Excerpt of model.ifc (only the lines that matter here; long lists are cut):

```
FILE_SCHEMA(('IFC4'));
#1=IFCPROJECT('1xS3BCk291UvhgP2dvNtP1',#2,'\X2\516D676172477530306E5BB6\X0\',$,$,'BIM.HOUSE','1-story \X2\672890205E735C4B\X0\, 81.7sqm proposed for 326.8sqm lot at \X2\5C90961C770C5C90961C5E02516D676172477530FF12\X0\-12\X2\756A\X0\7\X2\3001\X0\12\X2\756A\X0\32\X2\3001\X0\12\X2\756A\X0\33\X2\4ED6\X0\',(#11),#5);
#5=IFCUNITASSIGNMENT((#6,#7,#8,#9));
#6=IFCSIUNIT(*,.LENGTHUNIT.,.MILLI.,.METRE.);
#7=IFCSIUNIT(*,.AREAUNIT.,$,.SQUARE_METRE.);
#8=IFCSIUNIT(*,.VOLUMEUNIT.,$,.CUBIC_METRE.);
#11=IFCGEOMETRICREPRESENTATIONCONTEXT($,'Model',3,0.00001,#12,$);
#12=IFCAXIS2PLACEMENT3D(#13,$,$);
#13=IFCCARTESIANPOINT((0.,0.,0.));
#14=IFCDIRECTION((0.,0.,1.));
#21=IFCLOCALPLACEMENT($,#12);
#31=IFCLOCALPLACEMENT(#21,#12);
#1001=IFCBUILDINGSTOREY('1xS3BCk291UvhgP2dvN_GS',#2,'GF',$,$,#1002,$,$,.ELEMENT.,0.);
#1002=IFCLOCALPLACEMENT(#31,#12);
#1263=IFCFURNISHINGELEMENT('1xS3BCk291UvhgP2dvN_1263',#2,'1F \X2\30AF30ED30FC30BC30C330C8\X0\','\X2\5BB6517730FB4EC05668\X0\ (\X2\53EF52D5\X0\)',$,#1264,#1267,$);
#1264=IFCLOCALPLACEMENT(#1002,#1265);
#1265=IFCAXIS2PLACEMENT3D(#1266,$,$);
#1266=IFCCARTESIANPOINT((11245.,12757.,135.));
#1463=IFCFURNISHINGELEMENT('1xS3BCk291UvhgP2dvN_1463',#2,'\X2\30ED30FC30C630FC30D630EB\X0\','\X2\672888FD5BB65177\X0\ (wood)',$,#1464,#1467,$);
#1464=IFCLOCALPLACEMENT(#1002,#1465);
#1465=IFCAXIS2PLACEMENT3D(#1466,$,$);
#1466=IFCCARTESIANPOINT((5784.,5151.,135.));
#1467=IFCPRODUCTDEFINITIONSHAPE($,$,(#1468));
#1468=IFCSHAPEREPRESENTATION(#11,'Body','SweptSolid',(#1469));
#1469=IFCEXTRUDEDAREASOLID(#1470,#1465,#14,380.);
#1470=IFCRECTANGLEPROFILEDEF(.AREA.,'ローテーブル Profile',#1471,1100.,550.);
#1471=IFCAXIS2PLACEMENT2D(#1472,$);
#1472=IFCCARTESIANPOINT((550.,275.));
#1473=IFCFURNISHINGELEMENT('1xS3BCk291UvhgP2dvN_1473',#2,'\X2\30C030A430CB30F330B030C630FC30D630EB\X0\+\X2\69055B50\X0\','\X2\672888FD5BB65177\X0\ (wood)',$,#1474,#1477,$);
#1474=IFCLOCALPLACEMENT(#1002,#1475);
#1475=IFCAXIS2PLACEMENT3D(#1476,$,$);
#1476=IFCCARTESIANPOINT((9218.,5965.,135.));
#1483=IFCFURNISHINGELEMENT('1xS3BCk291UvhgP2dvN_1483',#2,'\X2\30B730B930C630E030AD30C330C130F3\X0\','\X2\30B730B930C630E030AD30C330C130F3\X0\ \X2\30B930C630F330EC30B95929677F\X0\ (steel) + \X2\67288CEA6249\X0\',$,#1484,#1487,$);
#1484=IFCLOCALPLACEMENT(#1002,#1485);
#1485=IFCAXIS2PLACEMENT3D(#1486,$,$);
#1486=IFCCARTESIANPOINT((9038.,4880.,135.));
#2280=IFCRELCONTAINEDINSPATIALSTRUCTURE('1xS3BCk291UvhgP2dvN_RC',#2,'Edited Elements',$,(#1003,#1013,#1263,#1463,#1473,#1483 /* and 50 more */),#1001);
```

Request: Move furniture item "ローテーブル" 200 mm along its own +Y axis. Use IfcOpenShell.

```python
import ifcopenshell
import ifcopenshell.api.geometry
import ifcopenshell.util.placement
import ifcopenshell.util.unit

model = ifcopenshell.open("model.ifc")
unit_scale = ifcopenshell.util.unit.calculate_unit_scale(model)

item = model.by_guid("1xS3BCk291UvhgP2dvN_1463")
matrix = ifcopenshell.util.placement.get_local_placement(item.ObjectPlacement)
matrix[:3, 3] += matrix[:3, 1] * 0.2 / unit_scale
ifcopenshell.api.geometry.edit_object_placement(model, product=item, matrix=matrix, is_si=False)

print(ifcopenshell.util.placement.get_local_placement(item.ObjectPlacement).round(3) + 0.0)

model.write("model_rev.ifc")
```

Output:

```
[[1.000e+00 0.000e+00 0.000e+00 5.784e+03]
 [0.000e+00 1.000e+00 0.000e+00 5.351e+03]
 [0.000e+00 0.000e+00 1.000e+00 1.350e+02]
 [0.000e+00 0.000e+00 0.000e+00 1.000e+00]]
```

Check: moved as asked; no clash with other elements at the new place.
